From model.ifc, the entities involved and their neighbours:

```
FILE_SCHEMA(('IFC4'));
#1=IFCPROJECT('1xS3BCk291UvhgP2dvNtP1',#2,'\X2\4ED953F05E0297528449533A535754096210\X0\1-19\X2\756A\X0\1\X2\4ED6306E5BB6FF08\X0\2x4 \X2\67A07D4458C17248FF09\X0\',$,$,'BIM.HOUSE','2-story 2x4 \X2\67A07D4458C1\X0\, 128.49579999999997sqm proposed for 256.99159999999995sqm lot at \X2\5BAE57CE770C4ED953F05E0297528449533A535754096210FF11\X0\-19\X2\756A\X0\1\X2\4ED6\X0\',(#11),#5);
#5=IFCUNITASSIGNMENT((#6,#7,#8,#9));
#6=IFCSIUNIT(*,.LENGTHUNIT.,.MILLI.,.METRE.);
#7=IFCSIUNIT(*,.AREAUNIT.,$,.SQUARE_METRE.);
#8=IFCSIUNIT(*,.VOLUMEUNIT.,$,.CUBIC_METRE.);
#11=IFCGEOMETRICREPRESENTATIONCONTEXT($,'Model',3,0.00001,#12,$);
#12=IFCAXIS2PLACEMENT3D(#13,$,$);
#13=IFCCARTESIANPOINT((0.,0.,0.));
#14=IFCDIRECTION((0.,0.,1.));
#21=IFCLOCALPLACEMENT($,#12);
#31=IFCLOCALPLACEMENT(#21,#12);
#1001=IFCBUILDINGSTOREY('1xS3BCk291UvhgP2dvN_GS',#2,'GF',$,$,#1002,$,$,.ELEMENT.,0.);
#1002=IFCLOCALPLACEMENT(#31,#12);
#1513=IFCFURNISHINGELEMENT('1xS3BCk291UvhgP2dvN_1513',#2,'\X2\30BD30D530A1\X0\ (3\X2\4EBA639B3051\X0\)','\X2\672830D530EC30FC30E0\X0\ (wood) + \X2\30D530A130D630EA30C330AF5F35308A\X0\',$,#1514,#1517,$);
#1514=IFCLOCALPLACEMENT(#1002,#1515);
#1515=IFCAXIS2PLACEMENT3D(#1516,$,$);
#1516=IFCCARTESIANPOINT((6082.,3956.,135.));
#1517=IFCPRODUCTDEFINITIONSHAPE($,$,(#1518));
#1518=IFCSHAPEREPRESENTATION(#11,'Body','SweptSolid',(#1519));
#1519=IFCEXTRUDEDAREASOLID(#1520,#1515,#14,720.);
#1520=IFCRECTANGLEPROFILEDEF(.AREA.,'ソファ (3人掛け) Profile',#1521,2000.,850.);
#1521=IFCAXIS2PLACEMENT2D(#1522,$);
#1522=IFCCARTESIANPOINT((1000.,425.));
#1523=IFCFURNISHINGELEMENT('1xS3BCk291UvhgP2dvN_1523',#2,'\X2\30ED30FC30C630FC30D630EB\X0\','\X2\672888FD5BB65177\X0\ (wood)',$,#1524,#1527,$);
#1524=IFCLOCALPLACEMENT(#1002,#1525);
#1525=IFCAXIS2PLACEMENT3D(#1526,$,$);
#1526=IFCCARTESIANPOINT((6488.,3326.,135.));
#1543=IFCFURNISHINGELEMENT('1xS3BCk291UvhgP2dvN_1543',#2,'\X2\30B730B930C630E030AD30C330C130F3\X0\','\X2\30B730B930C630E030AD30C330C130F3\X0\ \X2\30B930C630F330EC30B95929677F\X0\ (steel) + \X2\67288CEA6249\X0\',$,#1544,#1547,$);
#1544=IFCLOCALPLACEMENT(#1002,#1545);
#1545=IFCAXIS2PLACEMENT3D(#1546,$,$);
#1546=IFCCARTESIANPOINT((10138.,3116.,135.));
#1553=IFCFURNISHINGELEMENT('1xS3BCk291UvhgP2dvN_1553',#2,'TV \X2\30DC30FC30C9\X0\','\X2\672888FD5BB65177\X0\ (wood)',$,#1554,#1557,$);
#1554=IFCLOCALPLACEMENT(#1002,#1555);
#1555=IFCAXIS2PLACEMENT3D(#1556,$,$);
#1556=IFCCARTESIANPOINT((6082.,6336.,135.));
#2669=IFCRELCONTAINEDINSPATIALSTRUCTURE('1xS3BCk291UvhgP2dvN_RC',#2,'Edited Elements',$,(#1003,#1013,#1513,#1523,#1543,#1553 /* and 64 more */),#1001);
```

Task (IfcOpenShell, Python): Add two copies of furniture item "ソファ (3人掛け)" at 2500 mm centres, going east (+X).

```python
import numpy as np
import ifcopenshell
import ifcopenshell.api.geometry
import ifcopenshell.api.root
import ifcopenshell.util.element
import ifcopenshell.util.placement
import ifcopenshell.util.unit

model = ifcopenshell.open("model.ifc")
unit_scale = ifcopenshell.util.unit.calculate_unit_scale(model)


def reuse_history(source, copy):
    """copy_class also copies each property set's owner history, people and application; keep the originals."""
    for rel in copy.IsDefinedBy:
        if rel.is_a("IfcRelDefinesByProperties") and (history := rel.RelatingPropertyDefinition.OwnerHistory):
            rel.RelatingPropertyDefinition.OwnerHistory = source.OwnerHistory
            ifcopenshell.util.element.remove_deep2(model, history)


source = model.by_guid("1xS3BCk291UvhgP2dvN_1513")
base = ifcopenshell.util.placement.get_local_placement(source.ObjectPlacement)
step = np.array([1.0, 0.0, 0.0]) * 2.5 / unit_scale

for i in range(1, 3):
    copy = ifcopenshell.api.root.copy_class(model, product=source)
    copy.Representation = ifcopenshell.util.element.copy_deep(
        model, source.Representation, exclude=["IfcGeometricRepresentationContext", "IfcRepresentationMap"]
    )
    reuse_history(source, copy)
    matrix = base.copy()
    matrix[:3, 3] += i * step
    print("added at", matrix[:3, 3].round(3) + 0.0)
    ifcopenshell.api.geometry.edit_object_placement(model, product=copy, matrix=matrix, is_si=False)

model.write("model_updated.ifc")
```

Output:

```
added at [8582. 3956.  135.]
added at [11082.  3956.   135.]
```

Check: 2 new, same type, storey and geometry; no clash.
